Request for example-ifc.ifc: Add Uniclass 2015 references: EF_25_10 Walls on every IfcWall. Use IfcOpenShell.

First a look at what the model holds.

```python
import ifcopenshell

model = ifcopenshell.open("example-ifc.ifc")
print(model.schema)
print("classifications:", [c.Name for c in model.by_type("IfcClassification")])
for ifc_class in ("IfcDoor", "IfcRoof", "IfcStair", "IfcWall", "IfcWindow"):
    print(ifc_class, len(model.by_type(ifc_class)))
```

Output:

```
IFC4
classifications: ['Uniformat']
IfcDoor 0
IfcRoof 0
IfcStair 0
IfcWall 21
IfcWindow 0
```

```python
import ifcopenshell
import ifcopenshell.api.classification

model = ifcopenshell.open("example-ifc.ifc")

system = ifcopenshell.api.classification.add_classification(model, classification="Uniclass 2015")

codes = {
    "IfcWall": ("EF_25_10", "Walls"),
}
for ifc_class, (code, name) in codes.items():
    products = model.by_type(ifc_class)
    ifcopenshell.api.classification.add_reference(
        model, products=products, classification=system, identification=code, name=name
    )
    print(code, len(products))

model.write("example-ifc_edited.ifc")
```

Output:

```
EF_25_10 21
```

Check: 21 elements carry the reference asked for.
